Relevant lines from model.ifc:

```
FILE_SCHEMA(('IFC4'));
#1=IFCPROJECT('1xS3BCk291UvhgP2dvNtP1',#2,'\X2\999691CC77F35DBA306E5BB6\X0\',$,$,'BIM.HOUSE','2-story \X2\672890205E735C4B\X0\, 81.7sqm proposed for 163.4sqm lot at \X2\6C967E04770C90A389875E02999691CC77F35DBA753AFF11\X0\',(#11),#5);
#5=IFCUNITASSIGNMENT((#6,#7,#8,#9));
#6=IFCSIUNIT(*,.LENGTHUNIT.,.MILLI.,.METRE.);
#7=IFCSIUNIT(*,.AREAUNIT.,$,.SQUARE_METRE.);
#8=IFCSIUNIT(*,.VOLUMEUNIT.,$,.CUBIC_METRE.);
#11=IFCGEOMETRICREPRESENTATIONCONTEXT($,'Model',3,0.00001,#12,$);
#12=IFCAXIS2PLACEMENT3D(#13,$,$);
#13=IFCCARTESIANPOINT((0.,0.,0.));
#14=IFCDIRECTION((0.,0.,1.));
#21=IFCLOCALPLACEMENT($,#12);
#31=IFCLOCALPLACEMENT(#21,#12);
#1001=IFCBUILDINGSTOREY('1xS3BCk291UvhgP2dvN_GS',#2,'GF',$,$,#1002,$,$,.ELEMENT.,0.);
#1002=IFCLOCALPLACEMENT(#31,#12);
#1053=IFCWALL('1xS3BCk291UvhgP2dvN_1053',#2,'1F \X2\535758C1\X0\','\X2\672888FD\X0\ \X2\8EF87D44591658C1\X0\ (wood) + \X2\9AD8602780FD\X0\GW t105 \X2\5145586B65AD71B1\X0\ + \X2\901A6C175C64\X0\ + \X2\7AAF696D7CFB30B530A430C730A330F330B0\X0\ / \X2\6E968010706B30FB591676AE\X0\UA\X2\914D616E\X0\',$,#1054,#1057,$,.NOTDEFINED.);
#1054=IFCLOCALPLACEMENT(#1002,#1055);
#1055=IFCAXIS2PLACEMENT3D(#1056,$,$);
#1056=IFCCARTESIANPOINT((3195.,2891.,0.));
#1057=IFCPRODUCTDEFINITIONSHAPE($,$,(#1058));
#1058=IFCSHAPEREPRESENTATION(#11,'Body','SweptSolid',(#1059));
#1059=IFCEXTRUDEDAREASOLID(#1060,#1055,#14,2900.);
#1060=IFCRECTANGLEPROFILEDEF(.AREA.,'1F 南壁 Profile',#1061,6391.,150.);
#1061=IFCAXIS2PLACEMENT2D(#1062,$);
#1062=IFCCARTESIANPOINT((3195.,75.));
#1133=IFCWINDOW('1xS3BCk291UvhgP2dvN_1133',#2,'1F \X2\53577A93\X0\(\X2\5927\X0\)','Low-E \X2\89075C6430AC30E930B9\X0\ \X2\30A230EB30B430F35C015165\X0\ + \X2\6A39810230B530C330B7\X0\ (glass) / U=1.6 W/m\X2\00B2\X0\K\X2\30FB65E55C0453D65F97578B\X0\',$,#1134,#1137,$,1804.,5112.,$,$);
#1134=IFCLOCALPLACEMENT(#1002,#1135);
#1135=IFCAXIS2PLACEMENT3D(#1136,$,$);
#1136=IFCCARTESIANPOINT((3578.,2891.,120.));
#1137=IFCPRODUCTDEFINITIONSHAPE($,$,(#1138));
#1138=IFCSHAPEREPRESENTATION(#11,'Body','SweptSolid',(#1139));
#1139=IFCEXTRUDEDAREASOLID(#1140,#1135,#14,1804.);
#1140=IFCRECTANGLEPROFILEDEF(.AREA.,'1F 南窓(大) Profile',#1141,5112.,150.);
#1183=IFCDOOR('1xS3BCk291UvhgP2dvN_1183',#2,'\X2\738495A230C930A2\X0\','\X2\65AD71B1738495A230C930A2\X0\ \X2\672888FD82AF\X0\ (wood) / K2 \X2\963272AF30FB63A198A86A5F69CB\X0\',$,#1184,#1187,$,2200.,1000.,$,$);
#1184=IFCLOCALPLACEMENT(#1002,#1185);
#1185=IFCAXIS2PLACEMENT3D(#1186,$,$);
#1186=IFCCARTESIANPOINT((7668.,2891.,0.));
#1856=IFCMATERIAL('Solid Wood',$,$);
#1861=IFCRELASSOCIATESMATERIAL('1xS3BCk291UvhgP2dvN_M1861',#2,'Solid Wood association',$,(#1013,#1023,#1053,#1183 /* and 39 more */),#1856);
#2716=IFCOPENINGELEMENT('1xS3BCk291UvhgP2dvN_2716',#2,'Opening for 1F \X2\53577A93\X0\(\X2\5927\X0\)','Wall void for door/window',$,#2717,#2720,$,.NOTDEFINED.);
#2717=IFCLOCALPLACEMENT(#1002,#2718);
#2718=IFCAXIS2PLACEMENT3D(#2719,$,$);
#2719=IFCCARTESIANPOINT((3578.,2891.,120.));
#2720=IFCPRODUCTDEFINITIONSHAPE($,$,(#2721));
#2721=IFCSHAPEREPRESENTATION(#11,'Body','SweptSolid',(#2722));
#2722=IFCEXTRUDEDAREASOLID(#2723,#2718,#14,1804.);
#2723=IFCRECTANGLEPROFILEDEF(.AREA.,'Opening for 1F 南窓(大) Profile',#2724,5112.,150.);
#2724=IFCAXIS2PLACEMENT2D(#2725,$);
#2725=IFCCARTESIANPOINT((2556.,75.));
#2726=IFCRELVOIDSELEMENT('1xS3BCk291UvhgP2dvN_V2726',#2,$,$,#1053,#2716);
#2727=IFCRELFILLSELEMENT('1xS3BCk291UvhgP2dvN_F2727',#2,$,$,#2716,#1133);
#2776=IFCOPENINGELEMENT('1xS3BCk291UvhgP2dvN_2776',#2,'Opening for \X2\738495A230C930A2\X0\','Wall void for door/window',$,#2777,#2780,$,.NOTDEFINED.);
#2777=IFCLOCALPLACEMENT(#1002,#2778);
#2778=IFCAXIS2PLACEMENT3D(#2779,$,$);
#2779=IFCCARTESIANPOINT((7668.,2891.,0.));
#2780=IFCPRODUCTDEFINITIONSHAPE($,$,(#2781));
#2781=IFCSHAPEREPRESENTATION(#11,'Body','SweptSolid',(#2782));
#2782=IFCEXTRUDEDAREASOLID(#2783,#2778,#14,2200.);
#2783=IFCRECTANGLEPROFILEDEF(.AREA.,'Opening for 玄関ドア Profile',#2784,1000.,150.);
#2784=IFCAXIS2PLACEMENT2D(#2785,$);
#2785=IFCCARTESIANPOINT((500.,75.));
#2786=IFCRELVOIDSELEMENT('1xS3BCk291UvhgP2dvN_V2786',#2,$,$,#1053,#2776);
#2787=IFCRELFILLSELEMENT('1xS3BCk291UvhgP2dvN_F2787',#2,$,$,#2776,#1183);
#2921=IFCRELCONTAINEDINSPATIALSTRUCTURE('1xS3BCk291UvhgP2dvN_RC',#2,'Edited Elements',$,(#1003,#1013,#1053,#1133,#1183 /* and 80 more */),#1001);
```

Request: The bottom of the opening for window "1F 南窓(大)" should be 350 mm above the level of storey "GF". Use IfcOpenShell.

```python
import numpy as np
import ifcopenshell
import ifcopenshell.api.geometry
import ifcopenshell.geom
import ifcopenshell.util.element
import ifcopenshell.util.placement
import ifcopenshell.util.shape
import ifcopenshell.util.unit

model = ifcopenshell.open("model.ifc")
unit_scale = ifcopenshell.util.unit.calculate_unit_scale(model)

window = model.by_guid("1xS3BCk291UvhgP2dvN_1133")
opening = window.FillsVoids[0].RelatingOpeningElement
storey = ifcopenshell.util.element.get_container(window, ifc_class="IfcBuildingStorey")
level = ifcopenshell.util.placement.get_local_placement(storey.ObjectPlacement)[2, 3]

# The opening's origin need not be at the sill, so measure its lowest point.
shape = ifcopenshell.geom.create_shape(ifcopenshell.geom.settings(), opening)
bottom = ifcopenshell.util.shape.get_shape_bottom_elevation(shape, shape.geometry) / unit_scale
dz = level + 350.0 - bottom

shift = np.array([0.0, 0.0, dz])
# The window is not placed relative to its opening, so move both.
for product in (opening, window):
    matrix = ifcopenshell.util.placement.get_local_placement(product.ObjectPlacement)
    matrix[:3, 3] += shift
    ifcopenshell.api.geometry.edit_object_placement(model, product=product, matrix=matrix, is_si=False)

print(f"moved by {dz * unit_scale:+.3f} m")

model.write("model_updated.ifc")
```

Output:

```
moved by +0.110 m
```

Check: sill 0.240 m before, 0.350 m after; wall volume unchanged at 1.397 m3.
